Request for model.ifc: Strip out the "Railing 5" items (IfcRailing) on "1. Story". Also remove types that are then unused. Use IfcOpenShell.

First a look at what the model holds.

```python
import ifcopenshell
import ifcopenshell.util.element

model = ifcopenshell.open("model.ifc")
print(model.schema)
storey = next(s for s in model.by_type("IfcBuildingStorey") if s.Name == "1. Story")
railings = [e for e in ifcopenshell.util.element.get_decomposition(storey) if e.is_a("IfcRailing")]
seen = {}
for e in railings:
    element_type = ifcopenshell.util.element.get_type(e)
    name = element_type.Name if element_type not in (None, e) else None
    seen[name] = seen.get(name, 0) + 1
for name, count in sorted(seen.items(), key=str):
    print(count, "x", name)
```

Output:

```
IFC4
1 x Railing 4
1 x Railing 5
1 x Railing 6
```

```python
import ifcopenshell
import ifcopenshell.api.root
import ifcopenshell.util.element

model = ifcopenshell.open("model.ifc")

storey = next(s for s in model.by_type("IfcBuildingStorey") if s.Name == "1. Story")
railings = [e for e in ifcopenshell.util.element.get_decomposition(storey) if e.is_a("IfcRailing")]
targets = [e for e in railings if (t := ifcopenshell.util.element.get_type(e)) not in (None, e) and t.Name == "Railing 5"]
types = {ifcopenshell.util.element.get_type(e) for e in targets} - {None, *targets}

for e in targets:
    ifcopenshell.api.root.remove_product(model, product=e)
print(len(targets), "removed")

unused = [t for t in types if not ifcopenshell.util.element.get_types(t)]
for t in unused:
    ifcopenshell.api.root.remove_product(model, product=t)
print(len(unused), "unused types removed")

model.write("model_v2.ifc")
```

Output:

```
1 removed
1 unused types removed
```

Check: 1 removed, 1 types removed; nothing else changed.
